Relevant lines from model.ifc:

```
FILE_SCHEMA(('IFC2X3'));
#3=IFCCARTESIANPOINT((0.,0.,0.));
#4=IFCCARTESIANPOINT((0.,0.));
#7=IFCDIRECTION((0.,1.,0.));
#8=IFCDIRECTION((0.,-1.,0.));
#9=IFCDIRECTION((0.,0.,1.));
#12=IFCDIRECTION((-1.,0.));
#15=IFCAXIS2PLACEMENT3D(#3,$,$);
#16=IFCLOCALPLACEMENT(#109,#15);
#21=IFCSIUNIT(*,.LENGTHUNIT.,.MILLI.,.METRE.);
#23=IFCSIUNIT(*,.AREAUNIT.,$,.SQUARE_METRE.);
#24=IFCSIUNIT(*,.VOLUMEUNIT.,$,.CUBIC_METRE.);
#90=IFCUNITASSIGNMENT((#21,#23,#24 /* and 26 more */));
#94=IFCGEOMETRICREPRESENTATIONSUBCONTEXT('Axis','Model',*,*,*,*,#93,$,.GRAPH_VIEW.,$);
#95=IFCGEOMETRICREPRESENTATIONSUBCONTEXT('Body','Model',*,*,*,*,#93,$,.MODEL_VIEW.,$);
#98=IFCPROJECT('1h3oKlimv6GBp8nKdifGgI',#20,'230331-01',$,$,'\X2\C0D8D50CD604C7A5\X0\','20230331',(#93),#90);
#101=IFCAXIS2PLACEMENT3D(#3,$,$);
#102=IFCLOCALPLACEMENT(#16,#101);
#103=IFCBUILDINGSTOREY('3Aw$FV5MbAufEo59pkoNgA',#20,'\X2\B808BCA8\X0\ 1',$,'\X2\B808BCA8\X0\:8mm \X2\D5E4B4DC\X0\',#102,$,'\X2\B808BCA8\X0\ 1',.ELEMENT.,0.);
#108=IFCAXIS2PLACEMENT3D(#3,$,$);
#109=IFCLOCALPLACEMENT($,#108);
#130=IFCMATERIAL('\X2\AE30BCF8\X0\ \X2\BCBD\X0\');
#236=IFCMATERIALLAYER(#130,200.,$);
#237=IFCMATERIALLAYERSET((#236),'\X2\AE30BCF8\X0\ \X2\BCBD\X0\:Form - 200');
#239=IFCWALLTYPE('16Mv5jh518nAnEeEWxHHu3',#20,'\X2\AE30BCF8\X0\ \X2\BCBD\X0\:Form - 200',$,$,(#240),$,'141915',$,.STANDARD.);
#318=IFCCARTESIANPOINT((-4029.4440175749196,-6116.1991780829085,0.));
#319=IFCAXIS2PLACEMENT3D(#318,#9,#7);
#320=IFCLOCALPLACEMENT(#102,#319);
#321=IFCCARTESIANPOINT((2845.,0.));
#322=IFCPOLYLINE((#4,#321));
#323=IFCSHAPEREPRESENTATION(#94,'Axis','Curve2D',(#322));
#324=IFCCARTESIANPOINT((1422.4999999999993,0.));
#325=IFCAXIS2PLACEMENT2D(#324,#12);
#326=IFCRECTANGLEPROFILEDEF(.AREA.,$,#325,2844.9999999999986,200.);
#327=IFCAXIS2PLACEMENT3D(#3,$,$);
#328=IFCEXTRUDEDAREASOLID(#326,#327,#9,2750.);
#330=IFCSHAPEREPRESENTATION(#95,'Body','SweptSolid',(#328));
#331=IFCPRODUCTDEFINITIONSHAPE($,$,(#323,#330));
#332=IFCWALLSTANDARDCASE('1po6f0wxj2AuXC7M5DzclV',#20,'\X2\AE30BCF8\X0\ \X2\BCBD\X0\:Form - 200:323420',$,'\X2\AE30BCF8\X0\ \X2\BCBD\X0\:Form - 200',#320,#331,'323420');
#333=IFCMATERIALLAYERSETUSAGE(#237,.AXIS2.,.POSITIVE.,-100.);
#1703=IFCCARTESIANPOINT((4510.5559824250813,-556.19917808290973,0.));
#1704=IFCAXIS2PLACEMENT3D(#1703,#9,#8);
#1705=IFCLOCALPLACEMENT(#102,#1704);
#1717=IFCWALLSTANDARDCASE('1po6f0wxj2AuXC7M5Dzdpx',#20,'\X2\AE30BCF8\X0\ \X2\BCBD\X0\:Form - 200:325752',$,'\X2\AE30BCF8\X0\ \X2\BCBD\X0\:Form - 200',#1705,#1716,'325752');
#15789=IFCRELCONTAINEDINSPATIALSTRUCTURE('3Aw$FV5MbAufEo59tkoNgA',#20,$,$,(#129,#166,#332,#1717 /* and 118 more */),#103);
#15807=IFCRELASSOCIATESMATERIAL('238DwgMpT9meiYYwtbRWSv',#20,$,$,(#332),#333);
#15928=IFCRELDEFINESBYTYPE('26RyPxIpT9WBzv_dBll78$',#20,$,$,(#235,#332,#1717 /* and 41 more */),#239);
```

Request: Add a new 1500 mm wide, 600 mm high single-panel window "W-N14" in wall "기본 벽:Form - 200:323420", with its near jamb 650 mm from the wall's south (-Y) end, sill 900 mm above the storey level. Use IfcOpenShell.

```python
import numpy as np
import ifcopenshell
import ifcopenshell.api.feature
import ifcopenshell.api.geometry
import ifcopenshell.api.root
import ifcopenshell.api.spatial
import ifcopenshell.api.type
import ifcopenshell.geom
import ifcopenshell.util.element
import ifcopenshell.util.placement
import ifcopenshell.util.representation
import ifcopenshell.util.shape
import ifcopenshell.util.unit

model = ifcopenshell.open("model.ifc")
unit_scale = ifcopenshell.util.unit.calculate_unit_scale(model)
settings = ifcopenshell.geom.settings()


def volume(element):
    """Net volume in cubic metres, openings subtracted."""
    shape = ifcopenshell.geom.create_shape(settings, element)
    return ifcopenshell.util.shape.get_volume(shape.geometry)


wall = model.by_id(332)
storey = ifcopenshell.util.element.get_container(wall, ifc_class="IfcBuildingStorey")
context = ifcopenshell.util.representation.get_context(model, "Model", "Body", "MODEL_VIEW")
before = volume(wall)

width, height, from_end, sill = 1.5, 0.6, 0.65, 0.9  # metres

# The wall runs along its own X axis, and the end named is its -X end.
wall_shape = ifcopenshell.geom.create_shape(settings, wall)
x, y, z = ifcopenshell.util.shape.get_vertices(wall_shape.geometry).T
start = x.min() + from_end
face, thickness = float(y.min()), float(y.max() - y.min())
wall_matrix = ifcopenshell.util.placement.get_local_placement(wall.ObjectPlacement)
level = ifcopenshell.util.placement.get_local_placement(storey.ObjectPlacement)[2, 3]


def in_wall(x, y):
    """Placement at x, y metres in the wall's axes, at sill height."""
    matrix = wall_matrix.copy()
    matrix[:, 3] = wall_matrix @ np.array([x / unit_scale, y / unit_scale, 0.0, 1.0])
    matrix[2, 3] = level + sill / unit_scale
    return matrix


# Opening: a box that overshoots both wall faces by 50 mm.
opening = ifcopenshell.api.root.create_entity(model, ifc_class="IfcOpeningElement")
box = ifcopenshell.api.geometry.add_wall_representation(
    model, context=context, length=width, height=height, thickness=thickness + 0.1
)
ifcopenshell.api.geometry.assign_representation(model, product=opening, representation=box)
ifcopenshell.api.geometry.edit_object_placement(model, product=opening, matrix=in_wall(start, face - 0.05), is_si=False)
ifcopenshell.api.feature.add_feature(model, feature=opening, element=wall)

window = ifcopenshell.api.root.create_entity(model, ifc_class="IfcWindow", name="W-N14")
window.OverallWidth, window.OverallHeight = width / unit_scale, height / unit_scale
body = ifcopenshell.api.geometry.add_window_representation(
    model,
    context=context,
    overall_width=window.OverallWidth,
    overall_height=window.OverallHeight,
    partition_type="SINGLE_PANEL",
)
ifcopenshell.api.geometry.assign_representation(model, product=window, representation=body)
ifcopenshell.api.spatial.assign_container(model, products=[window], relating_structure=storey)
fills = ifcopenshell.api.feature.add_filling(model, opening=opening, element=window)
fills.OwnerHistory = window.OwnerHistory  # required in IFC2X3

# IFC2X3 keeps the operation on the window style.
style = ifcopenshell.api.root.create_entity(model, ifc_class="IfcWindowStyle", name="W-N14")
style.OperationType, style.ConstructionType = "SINGLE_PANEL", "NOTDEFINED"
style.ParameterTakesPrecedence = style.Sizeable = False
ifcopenshell.api.type.assign_type(model, related_objects=[window], relating_type=style)

# Centre the window in the wall's thickness.
ifcopenshell.api.geometry.edit_object_placement(model, product=window, matrix=in_wall(start, face), is_si=False)
window_shape = ifcopenshell.geom.create_shape(settings, window)
depth = ifcopenshell.util.shape.get_vertices(window_shape.geometry)[:, 1]
offset = face + thickness / 2 - (depth.min() + depth.max()) / 2
ifcopenshell.api.geometry.edit_object_placement(model, product=window, matrix=in_wall(start, offset), is_si=False)

after = volume(wall)

print(f"wall volume {before:.3f} -> {after:.3f} m3")

model.write("model_rev.ifc")
```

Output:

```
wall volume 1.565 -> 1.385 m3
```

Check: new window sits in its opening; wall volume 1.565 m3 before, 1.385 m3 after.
